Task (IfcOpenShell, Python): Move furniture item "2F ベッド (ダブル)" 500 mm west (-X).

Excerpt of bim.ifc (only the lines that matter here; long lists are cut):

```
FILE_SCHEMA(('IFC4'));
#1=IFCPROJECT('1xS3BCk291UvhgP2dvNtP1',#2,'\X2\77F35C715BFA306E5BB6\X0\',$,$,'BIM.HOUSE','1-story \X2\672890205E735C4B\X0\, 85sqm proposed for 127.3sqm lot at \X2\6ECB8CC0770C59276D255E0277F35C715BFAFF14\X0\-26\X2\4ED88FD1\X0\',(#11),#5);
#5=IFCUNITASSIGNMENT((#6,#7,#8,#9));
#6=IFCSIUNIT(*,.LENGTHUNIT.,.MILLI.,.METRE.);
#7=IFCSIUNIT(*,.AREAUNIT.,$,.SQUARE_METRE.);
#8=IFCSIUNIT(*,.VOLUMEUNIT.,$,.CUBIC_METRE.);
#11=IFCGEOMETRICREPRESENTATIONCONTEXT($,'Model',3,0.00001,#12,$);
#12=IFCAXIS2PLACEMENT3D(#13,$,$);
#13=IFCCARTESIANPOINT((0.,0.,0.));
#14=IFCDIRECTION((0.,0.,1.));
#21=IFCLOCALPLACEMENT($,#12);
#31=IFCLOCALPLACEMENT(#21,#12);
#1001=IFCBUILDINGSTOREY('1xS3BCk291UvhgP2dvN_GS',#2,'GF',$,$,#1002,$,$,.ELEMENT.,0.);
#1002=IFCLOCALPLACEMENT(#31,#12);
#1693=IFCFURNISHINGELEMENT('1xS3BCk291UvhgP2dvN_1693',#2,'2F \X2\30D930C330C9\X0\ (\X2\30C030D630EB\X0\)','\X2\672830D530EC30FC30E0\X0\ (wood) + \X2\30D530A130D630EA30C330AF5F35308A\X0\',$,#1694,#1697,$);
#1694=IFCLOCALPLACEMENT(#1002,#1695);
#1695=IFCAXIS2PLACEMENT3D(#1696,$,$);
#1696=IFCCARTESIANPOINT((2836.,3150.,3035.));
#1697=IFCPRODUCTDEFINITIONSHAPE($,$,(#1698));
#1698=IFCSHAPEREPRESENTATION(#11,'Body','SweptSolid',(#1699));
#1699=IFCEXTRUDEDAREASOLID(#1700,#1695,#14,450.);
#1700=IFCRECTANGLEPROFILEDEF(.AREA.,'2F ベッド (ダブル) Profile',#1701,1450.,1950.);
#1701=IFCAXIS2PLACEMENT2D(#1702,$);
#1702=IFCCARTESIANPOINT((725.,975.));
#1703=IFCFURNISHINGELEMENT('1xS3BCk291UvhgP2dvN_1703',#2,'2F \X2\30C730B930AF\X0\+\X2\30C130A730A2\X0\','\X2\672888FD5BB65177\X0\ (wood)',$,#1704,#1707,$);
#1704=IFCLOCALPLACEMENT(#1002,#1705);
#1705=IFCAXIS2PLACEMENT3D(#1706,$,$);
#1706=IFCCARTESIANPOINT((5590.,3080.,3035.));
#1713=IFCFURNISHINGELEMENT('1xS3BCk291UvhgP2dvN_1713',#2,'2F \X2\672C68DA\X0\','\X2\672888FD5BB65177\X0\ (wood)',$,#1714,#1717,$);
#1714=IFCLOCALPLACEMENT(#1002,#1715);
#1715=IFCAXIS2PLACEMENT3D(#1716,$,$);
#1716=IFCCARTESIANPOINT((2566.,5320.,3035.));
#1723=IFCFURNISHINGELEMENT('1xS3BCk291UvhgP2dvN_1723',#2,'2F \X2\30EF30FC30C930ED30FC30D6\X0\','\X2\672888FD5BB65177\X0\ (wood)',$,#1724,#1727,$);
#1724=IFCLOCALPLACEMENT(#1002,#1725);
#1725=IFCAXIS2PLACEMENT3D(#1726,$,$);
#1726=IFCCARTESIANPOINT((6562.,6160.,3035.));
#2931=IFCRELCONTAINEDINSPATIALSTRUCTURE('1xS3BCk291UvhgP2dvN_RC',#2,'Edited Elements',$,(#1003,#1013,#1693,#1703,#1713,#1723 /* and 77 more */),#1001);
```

```python
import ifcopenshell
import ifcopenshell.api.geometry
import ifcopenshell.util.placement
import ifcopenshell.util.unit

model = ifcopenshell.open("bim.ifc")
unit_scale = ifcopenshell.util.unit.calculate_unit_scale(model)

item = model.by_guid("1xS3BCk291UvhgP2dvN_1693")
matrix = ifcopenshell.util.placement.get_local_placement(item.ObjectPlacement)
matrix[0, 3] -= 0.5 / unit_scale
ifcopenshell.api.geometry.edit_object_placement(model, product=item, matrix=matrix, is_si=False)

print(ifcopenshell.util.placement.get_local_placement(item.ObjectPlacement).round(3) + 0.0)

model.write("bim-out.ifc")
```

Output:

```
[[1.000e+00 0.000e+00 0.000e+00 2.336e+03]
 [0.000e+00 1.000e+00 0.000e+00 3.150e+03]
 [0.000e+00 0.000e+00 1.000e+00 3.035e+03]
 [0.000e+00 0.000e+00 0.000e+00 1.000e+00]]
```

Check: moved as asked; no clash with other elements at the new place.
